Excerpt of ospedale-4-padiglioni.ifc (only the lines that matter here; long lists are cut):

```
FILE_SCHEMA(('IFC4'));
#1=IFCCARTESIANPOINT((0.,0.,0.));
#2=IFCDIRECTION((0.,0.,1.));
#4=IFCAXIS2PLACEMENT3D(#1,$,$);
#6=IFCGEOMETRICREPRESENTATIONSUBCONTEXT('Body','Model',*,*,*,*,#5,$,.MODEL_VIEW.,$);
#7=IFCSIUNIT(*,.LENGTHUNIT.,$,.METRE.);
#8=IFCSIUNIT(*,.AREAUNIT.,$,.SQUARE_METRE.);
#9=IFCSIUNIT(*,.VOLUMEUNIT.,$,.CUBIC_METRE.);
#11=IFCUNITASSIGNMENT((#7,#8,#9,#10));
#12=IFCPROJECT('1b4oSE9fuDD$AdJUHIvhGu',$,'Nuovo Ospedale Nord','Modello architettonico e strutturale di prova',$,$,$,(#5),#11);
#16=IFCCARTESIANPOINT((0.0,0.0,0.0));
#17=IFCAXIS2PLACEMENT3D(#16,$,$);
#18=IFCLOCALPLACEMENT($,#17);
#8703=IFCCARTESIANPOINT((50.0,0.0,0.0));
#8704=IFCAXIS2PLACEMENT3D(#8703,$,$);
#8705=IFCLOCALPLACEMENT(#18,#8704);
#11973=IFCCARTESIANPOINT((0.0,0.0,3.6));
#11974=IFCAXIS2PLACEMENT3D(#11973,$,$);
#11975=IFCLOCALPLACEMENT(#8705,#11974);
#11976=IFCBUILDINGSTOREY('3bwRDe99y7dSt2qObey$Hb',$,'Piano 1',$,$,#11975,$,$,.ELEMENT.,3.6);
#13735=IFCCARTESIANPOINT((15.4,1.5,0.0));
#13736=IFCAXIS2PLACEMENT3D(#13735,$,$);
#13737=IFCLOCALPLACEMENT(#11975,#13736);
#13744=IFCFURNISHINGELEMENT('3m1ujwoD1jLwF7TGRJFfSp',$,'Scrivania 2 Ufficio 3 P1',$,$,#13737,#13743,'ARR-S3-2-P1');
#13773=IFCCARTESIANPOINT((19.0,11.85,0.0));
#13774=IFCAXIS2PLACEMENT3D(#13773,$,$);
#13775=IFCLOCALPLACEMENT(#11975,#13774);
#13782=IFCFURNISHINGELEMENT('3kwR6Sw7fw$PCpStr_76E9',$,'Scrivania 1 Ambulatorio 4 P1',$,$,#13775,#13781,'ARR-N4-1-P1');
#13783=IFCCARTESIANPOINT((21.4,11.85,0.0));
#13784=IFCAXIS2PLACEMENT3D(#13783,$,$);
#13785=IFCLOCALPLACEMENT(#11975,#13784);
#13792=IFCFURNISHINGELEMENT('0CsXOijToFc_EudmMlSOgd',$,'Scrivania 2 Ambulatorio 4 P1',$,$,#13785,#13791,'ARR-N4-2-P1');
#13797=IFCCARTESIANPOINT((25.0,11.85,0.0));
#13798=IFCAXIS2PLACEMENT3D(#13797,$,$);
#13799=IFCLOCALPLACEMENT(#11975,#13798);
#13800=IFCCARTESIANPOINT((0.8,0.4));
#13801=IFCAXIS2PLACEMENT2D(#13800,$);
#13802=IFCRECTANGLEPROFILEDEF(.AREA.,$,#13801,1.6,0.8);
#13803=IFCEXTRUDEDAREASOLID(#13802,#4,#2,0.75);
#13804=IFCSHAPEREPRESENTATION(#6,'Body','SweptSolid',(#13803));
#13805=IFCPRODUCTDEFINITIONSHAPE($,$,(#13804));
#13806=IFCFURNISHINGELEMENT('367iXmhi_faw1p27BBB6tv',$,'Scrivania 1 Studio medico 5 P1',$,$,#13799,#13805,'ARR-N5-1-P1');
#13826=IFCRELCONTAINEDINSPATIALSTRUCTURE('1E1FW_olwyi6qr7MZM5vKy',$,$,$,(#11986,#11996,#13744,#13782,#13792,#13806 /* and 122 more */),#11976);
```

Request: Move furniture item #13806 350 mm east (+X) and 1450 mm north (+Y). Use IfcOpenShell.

```python
import ifcopenshell
import ifcopenshell.api.geometry
import ifcopenshell.util.placement

model = ifcopenshell.open("ospedale-4-padiglioni.ifc")

item = model.by_id(13806)
matrix = ifcopenshell.util.placement.get_local_placement(item.ObjectPlacement)
matrix[0, 3] += 0.35
matrix[1, 3] += 1.45
ifcopenshell.api.geometry.edit_object_placement(model, product=item, matrix=matrix, is_si=False)

print(ifcopenshell.util.placement.get_local_placement(item.ObjectPlacement).round(3) + 0.0)

model.write("ospedale-4-padiglioni_v2.ifc")
```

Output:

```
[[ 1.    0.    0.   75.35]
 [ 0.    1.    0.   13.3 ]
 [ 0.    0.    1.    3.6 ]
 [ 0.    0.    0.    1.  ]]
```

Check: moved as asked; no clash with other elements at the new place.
